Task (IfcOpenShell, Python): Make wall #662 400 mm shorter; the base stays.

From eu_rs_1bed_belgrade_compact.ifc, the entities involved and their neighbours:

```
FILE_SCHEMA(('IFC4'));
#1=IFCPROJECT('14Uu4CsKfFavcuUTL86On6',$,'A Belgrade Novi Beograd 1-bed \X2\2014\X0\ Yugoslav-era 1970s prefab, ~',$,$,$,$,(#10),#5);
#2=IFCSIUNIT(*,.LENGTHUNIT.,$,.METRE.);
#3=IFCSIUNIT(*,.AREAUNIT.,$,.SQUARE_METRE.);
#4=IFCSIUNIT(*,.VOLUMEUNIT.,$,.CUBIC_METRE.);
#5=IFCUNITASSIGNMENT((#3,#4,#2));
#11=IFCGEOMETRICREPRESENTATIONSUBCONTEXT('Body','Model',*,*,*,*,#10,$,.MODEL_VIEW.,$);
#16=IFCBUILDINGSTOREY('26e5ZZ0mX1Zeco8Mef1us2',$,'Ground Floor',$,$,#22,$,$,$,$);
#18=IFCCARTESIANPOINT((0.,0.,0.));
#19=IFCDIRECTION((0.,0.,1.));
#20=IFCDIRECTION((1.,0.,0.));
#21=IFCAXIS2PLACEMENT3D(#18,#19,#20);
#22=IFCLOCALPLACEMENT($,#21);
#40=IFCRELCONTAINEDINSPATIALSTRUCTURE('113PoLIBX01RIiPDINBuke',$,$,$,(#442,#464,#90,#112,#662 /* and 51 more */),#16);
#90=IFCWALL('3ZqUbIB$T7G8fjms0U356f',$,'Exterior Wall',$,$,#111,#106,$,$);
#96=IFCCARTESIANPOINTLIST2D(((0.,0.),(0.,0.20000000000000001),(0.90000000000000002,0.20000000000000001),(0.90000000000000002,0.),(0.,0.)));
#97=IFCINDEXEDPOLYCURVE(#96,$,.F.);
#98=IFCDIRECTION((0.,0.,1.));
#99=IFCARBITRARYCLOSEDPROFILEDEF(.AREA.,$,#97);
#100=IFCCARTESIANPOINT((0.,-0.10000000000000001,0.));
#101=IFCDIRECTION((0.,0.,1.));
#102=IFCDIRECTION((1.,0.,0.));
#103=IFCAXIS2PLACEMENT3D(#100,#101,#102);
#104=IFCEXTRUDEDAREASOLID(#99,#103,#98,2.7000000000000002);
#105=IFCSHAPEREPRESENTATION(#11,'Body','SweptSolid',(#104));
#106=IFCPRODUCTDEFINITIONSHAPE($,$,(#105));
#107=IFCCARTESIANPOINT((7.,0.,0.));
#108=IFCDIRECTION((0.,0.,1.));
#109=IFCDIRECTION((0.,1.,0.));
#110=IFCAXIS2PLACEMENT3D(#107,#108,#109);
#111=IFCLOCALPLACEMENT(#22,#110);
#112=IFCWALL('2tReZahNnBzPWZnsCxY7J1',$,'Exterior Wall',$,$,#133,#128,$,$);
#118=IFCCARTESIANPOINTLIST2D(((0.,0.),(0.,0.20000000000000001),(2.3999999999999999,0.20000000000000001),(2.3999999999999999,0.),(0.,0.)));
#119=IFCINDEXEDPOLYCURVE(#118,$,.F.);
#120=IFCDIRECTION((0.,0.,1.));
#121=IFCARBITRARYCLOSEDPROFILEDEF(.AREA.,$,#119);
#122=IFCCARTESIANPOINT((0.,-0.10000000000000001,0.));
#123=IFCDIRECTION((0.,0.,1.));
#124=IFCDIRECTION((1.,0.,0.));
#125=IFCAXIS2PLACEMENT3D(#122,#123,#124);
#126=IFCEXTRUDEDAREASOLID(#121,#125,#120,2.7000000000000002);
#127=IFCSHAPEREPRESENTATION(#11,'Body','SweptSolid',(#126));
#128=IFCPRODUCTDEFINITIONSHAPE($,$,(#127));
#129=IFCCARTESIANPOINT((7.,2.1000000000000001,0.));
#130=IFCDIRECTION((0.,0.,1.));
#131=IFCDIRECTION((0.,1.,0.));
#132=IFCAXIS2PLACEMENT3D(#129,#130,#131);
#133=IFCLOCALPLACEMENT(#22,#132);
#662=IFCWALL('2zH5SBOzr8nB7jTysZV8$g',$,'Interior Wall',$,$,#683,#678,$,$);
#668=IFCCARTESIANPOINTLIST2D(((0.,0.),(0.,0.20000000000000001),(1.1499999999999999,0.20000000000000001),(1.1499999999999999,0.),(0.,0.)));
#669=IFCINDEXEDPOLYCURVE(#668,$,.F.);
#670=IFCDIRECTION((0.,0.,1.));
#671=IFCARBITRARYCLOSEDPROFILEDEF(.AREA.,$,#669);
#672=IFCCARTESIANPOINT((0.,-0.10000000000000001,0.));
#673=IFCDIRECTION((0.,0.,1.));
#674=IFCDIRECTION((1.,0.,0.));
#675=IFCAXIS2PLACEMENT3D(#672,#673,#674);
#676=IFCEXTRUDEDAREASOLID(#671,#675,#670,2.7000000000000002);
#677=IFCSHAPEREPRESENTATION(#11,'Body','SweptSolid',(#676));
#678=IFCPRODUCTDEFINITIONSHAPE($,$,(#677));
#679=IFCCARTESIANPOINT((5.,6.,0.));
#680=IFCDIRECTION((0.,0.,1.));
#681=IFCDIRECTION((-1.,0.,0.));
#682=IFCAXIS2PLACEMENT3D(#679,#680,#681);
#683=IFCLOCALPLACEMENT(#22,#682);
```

```python
import ifcopenshell
import ifcopenshell.geom
import ifcopenshell.util.representation
import ifcopenshell.util.shape
import ifcopenshell.util.unit

model = ifcopenshell.open("eu_rs_1bed_belgrade_compact.ifc")
unit_scale = ifcopenshell.util.unit.calculate_unit_scale(model)
settings = ifcopenshell.geom.settings()


def volume(element):
    """Net volume in cubic metres, openings subtracted."""
    shape = ifcopenshell.geom.create_shape(settings, element)
    return ifcopenshell.util.shape.get_volume(shape.geometry)


wall = model.by_id(662)
before = volume(wall)

body = ifcopenshell.util.representation.get_representation(wall, "Model", "Body")
solid = body.Items[0]
old_height = solid.Depth
solid.Depth -= 0.4 / unit_scale
after = volume(wall)

print(f"height {old_height:g} -> {solid.Depth:g}, volume {before:.3f} -> {after:.3f} m3")

model.write("eu_rs_1bed_belgrade_compact_updated.ifc")
```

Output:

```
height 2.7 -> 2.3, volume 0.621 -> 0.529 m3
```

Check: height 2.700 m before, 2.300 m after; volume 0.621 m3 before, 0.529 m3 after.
